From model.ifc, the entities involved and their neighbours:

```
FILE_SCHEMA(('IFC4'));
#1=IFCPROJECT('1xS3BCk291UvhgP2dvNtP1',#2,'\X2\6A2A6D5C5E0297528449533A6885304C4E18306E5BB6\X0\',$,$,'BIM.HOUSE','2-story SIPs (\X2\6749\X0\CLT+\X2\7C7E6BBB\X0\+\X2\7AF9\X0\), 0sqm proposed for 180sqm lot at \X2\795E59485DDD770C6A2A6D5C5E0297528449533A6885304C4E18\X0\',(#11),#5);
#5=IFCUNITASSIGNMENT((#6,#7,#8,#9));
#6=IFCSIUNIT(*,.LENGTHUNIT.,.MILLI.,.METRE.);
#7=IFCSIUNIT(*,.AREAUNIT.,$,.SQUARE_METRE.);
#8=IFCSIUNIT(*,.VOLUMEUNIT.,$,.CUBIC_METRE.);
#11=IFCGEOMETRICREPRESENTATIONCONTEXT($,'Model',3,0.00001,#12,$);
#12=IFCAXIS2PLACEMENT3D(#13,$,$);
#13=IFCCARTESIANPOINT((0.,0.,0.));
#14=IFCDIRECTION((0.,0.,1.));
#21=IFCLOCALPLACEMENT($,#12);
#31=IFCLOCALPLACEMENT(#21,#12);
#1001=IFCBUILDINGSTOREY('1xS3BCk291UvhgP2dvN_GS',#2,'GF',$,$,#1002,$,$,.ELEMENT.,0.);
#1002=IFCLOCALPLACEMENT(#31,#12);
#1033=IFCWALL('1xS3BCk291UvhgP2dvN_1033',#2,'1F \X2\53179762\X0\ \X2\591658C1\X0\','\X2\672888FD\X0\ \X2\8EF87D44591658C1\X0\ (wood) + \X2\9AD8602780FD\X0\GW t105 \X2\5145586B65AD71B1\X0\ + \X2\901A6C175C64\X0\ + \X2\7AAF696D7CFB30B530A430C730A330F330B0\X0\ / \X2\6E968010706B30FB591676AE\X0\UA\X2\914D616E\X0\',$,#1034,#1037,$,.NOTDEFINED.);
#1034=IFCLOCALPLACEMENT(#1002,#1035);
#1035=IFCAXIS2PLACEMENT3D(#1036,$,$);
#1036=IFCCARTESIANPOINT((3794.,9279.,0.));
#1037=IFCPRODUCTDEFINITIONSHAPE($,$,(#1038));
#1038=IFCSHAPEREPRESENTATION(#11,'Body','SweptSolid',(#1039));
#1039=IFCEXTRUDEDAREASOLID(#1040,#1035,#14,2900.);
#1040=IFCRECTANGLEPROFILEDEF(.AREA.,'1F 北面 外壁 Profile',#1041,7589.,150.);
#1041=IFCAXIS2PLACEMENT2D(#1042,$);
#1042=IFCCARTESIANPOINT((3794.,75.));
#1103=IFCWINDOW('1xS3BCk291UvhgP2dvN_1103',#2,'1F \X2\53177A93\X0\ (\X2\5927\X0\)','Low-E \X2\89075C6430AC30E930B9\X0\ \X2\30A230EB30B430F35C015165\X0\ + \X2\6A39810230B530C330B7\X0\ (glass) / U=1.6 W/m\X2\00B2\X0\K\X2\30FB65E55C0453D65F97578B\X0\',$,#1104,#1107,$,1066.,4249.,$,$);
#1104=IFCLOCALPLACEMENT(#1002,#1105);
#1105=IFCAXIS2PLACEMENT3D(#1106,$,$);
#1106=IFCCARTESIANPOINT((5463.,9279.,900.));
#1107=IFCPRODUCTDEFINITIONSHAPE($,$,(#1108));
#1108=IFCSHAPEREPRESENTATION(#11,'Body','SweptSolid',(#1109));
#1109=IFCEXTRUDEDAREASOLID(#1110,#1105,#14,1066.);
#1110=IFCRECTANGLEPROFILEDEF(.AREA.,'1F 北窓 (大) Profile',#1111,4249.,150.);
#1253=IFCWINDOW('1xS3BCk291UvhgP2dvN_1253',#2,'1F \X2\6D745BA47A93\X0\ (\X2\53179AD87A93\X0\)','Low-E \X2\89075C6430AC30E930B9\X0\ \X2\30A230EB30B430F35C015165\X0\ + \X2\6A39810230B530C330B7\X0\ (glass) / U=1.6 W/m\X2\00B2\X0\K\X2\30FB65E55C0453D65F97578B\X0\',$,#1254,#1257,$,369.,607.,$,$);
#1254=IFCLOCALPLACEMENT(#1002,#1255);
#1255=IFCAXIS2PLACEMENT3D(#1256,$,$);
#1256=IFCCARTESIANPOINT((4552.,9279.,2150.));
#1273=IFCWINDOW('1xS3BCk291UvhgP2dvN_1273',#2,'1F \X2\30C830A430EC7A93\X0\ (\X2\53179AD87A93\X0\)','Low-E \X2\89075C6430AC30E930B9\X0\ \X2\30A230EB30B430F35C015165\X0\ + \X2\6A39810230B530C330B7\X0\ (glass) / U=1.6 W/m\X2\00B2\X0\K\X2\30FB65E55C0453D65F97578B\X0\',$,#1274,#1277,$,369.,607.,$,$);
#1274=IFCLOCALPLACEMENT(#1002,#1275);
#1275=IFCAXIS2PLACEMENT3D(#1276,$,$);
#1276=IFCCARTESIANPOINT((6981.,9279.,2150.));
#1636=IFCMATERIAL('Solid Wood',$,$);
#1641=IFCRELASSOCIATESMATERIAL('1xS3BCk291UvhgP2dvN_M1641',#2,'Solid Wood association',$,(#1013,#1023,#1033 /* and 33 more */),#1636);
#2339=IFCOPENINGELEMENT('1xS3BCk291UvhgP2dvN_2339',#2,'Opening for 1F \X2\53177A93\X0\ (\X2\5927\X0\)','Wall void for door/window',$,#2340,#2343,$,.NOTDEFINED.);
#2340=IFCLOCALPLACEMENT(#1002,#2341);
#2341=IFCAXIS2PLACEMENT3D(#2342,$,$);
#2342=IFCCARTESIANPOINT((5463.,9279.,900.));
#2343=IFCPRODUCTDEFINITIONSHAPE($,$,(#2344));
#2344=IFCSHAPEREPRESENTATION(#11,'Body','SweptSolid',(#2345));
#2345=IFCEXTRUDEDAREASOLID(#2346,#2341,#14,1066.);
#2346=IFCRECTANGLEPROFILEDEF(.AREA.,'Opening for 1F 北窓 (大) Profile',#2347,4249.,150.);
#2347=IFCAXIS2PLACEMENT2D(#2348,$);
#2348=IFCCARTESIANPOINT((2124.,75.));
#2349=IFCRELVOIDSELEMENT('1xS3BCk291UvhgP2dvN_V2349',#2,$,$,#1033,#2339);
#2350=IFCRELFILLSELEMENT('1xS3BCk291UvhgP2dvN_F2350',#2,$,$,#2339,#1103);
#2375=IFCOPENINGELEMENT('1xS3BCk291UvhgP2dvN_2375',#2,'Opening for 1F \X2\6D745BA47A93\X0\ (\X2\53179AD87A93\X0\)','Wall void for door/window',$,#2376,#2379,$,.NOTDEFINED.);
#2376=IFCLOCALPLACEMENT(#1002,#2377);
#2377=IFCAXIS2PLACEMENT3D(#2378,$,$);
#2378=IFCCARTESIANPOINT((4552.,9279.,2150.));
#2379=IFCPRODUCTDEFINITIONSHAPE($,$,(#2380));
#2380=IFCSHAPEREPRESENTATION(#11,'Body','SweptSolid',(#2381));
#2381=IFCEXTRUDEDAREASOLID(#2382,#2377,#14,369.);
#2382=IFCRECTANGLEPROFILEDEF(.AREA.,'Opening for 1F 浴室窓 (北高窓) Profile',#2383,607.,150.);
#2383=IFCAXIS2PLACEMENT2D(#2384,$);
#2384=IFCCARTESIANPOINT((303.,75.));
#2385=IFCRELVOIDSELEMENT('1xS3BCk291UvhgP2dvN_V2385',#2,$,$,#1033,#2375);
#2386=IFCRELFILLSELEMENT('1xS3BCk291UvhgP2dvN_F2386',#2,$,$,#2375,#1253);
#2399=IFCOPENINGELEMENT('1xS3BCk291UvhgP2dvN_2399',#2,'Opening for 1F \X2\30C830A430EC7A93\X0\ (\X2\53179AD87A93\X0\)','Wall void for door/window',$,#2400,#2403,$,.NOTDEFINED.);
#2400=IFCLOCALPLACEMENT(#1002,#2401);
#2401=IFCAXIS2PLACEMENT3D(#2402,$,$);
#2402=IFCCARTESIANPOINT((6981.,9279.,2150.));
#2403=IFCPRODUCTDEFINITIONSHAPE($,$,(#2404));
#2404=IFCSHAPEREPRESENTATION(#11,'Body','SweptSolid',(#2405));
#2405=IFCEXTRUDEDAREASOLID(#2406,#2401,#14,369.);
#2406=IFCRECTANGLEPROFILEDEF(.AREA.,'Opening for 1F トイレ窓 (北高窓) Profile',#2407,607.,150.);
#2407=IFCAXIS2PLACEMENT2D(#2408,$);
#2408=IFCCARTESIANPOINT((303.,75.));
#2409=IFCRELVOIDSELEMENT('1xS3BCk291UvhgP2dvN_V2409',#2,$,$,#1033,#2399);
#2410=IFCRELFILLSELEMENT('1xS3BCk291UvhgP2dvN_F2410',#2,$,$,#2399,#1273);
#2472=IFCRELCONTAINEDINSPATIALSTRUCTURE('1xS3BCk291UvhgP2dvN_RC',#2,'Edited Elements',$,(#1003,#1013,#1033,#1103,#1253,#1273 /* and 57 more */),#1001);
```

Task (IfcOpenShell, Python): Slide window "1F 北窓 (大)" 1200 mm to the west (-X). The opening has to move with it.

```python
import ifcopenshell
import ifcopenshell.api.geometry
import ifcopenshell.util.placement

model = ifcopenshell.open("model.ifc")

window = model.by_id(1103)
opening = window.FillsVoids[0].RelatingOpeningElement
wall = opening.VoidsElements[0].RelatingBuildingElement

wall_matrix = ifcopenshell.util.placement.get_local_placement(wall.ObjectPlacement)
shift = wall_matrix[:3, 0] * -1200.0
before = ifcopenshell.util.placement.get_local_placement(window.ObjectPlacement)[:3, 3].copy()

# The window is not placed relative to its opening, so move both.
for product in (opening, window):
    matrix = ifcopenshell.util.placement.get_local_placement(product.ObjectPlacement)
    matrix[:3, 3] += shift
    ifcopenshell.api.geometry.edit_object_placement(model, product=product, matrix=matrix, is_si=False)

after = ifcopenshell.util.placement.get_local_placement(window.ObjectPlacement)[:3, 3]
print("window moved by", (after - before).round(3) + 0.0)

model.write("model_updated.ifc")
```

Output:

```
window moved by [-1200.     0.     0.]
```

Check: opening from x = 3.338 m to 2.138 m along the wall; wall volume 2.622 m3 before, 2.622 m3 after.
